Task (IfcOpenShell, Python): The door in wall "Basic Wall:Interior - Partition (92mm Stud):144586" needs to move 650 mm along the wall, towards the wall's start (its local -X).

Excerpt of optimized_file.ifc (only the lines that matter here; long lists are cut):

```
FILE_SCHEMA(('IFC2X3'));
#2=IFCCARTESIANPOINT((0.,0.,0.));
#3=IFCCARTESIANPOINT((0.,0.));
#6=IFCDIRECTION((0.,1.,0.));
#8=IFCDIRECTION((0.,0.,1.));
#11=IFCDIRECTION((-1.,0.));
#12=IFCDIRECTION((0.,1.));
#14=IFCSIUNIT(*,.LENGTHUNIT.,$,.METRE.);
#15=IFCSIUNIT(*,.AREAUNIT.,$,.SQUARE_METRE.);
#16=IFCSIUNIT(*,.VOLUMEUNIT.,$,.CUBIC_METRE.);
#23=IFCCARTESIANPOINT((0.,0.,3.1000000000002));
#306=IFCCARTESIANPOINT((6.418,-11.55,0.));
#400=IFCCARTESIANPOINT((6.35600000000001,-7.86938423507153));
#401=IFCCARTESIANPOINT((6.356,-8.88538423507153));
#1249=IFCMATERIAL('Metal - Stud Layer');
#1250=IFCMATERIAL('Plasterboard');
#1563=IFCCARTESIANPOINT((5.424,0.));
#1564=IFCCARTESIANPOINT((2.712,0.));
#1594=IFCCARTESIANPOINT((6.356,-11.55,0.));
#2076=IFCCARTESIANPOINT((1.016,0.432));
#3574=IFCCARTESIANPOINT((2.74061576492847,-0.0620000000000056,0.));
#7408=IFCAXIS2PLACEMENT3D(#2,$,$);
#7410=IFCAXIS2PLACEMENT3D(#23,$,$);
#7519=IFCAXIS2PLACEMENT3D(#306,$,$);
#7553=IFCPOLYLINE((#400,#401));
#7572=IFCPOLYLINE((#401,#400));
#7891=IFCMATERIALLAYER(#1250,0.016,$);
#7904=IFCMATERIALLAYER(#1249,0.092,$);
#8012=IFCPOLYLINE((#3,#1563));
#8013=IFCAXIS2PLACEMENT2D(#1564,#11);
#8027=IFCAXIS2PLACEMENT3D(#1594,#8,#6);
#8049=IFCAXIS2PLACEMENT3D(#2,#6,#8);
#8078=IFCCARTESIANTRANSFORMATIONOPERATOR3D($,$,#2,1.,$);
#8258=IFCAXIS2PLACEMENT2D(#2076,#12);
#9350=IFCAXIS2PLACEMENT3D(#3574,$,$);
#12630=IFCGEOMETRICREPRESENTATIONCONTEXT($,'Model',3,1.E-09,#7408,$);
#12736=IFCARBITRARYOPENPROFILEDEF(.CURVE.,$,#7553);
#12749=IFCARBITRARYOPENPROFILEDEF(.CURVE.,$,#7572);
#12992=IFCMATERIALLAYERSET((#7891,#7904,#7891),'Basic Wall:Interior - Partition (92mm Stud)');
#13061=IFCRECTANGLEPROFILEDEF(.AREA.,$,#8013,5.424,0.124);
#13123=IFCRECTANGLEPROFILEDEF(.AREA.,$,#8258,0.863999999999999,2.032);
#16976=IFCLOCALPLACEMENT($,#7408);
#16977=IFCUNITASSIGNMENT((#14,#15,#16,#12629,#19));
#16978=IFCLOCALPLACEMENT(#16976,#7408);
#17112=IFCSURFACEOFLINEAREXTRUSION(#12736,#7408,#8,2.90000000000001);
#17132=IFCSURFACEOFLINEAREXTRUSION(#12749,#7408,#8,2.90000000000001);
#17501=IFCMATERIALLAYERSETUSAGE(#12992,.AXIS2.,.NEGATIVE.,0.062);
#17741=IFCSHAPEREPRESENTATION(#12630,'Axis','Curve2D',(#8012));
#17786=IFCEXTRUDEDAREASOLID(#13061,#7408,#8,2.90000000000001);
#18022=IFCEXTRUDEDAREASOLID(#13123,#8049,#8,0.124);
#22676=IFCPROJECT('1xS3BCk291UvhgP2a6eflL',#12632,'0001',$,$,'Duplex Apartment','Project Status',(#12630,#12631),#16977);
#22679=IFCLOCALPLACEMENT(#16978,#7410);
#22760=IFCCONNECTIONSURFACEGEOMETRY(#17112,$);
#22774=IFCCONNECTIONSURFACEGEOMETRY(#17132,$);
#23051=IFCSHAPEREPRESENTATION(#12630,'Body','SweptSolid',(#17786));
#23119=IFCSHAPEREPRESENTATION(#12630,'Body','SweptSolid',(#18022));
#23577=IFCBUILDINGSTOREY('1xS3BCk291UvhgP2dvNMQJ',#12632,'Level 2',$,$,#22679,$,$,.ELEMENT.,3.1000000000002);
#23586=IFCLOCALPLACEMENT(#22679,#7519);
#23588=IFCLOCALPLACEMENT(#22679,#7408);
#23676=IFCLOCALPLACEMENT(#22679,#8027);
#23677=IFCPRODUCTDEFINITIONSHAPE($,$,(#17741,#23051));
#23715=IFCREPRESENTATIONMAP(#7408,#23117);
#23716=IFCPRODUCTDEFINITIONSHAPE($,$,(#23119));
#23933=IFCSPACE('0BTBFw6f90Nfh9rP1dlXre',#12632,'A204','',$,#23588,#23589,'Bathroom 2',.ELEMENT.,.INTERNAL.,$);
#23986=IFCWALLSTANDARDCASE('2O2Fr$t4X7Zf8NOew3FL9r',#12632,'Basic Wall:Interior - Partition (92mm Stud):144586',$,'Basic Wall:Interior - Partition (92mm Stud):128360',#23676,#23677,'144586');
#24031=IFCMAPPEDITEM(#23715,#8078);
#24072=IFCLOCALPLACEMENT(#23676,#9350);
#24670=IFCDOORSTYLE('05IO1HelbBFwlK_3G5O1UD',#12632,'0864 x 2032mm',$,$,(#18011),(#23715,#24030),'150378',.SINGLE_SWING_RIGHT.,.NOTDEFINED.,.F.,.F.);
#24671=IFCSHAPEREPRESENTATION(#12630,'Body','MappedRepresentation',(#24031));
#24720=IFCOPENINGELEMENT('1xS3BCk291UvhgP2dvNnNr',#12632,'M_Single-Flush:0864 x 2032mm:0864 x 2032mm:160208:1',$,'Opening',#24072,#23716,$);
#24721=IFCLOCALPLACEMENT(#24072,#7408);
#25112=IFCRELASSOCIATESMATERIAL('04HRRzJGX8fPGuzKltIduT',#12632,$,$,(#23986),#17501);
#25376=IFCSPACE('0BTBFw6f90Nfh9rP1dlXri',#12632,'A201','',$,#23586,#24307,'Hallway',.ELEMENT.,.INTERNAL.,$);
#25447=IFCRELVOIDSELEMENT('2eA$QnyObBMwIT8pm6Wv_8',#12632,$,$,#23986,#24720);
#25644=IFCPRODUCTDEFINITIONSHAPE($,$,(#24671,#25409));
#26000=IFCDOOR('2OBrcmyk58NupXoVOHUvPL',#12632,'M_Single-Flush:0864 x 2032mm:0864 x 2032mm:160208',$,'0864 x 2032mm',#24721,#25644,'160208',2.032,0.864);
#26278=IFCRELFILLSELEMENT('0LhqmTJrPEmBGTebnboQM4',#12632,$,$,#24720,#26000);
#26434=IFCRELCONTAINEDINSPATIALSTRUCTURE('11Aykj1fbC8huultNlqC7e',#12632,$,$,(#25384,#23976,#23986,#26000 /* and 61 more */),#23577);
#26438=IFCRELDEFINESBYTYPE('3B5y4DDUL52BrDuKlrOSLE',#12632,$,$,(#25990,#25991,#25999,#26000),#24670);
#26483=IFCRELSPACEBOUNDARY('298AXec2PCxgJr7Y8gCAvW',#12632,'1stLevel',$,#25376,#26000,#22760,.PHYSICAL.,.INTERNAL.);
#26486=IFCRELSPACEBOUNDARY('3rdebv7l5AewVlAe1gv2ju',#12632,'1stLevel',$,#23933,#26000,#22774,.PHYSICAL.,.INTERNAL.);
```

```python
import numpy as np
import ifcopenshell
import ifcopenshell.api.geometry
import ifcopenshell.util.placement
import ifcopenshell.util.unit

model = ifcopenshell.open("optimized_file.ifc")
unit_scale = ifcopenshell.util.unit.calculate_unit_scale(model)

door = model.by_id(26000)
opening = door.FillsVoids[0].RelatingOpeningElement
wall = opening.VoidsElements[0].RelatingBuildingElement

wall_matrix = ifcopenshell.util.placement.get_local_placement(wall.ObjectPlacement)
shift = wall_matrix[:3, 0] * -0.65 / unit_scale
before = ifcopenshell.util.placement.get_local_placement(door.ObjectPlacement)[:3, 3].copy()

# The door is placed relative to its opening, so it follows when the opening moves.
matrix = ifcopenshell.util.placement.get_local_placement(opening.ObjectPlacement)
matrix[:3, 3] += shift
ifcopenshell.api.geometry.edit_object_placement(
    model, product=opening, matrix=matrix, is_si=False, should_transform_children=True
)

# Space boundary surfaces are stored in each space's coordinates; move them too.
for rel in door.ProvidesBoundaries:
    if not rel.ConnectionGeometry:
        continue
    surface = rel.ConnectionGeometry.SurfaceOnRelatingElement
    space_matrix = ifcopenshell.util.placement.get_local_placement(rel.RelatingSpace.ObjectPlacement)
    point = np.array(surface.Position.Location.Coordinates) + space_matrix[:3, :3].T @ shift
    surface.Position = model.createIfcAxis2Placement3D(
        model.createIfcCartesianPoint(point.tolist()), surface.Position.Axis, surface.Position.RefDirection
    )

after = ifcopenshell.util.placement.get_local_placement(door.ObjectPlacement)[:3, 3]
print("door moved by", (after - before).round(3) + 0.0)

model.write("optimized_file_edited.ifc")
```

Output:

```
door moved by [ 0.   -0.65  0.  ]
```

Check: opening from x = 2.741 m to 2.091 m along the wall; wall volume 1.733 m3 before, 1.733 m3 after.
